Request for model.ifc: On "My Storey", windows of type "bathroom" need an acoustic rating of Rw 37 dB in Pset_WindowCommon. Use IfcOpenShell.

First a look at what the model holds.

```python
import ifcopenshell
import ifcopenshell.util.element

model = ifcopenshell.open("model.ifc")
print(model.schema)
storey = next(s for s in model.by_type("IfcBuildingStorey") if s.Name == "My Storey")
windows = [e for e in ifcopenshell.util.element.get_decomposition(storey) if e.is_a("IfcWindow")]
seen = {}
for e in windows:
    element_type = ifcopenshell.util.element.get_type(e)
    key = (element_type.Name if element_type != e and element_type else None, ifcopenshell.util.element.get_pset(e, "Pset_WindowCommon", "AcousticRating"))
    seen[key] = seen.get(key, 0) + 1
for (name, value), count in sorted(seen.items(), key=str):
    print(count, "x", name, "|", value)
```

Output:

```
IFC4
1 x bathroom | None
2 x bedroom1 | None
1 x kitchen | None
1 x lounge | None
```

```python
import ifcopenshell
import ifcopenshell.api.pset
import ifcopenshell.util.element

model = ifcopenshell.open("model.ifc")

storey = next(s for s in model.by_type("IfcBuildingStorey") if s.Name == "My Storey")
windows = [e for e in ifcopenshell.util.element.get_decomposition(storey) if e.is_a("IfcWindow")]

count = 0
for e in windows:
    element_type = ifcopenshell.util.element.get_type(e)
    if element_type in (None, e) or element_type.Name != "bathroom":
        continue
    # add_pset returns the element's existing set when there is one.
    pset = ifcopenshell.api.pset.add_pset(model, product=e, name="Pset_WindowCommon")
    ifcopenshell.api.pset.edit_pset(model, pset=pset, properties={"AcousticRating": "Rw 37 dB"})
    count += 1

print(count, "windows updated")

model.write("model_v2.ifc")
```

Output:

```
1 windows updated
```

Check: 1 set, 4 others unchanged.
